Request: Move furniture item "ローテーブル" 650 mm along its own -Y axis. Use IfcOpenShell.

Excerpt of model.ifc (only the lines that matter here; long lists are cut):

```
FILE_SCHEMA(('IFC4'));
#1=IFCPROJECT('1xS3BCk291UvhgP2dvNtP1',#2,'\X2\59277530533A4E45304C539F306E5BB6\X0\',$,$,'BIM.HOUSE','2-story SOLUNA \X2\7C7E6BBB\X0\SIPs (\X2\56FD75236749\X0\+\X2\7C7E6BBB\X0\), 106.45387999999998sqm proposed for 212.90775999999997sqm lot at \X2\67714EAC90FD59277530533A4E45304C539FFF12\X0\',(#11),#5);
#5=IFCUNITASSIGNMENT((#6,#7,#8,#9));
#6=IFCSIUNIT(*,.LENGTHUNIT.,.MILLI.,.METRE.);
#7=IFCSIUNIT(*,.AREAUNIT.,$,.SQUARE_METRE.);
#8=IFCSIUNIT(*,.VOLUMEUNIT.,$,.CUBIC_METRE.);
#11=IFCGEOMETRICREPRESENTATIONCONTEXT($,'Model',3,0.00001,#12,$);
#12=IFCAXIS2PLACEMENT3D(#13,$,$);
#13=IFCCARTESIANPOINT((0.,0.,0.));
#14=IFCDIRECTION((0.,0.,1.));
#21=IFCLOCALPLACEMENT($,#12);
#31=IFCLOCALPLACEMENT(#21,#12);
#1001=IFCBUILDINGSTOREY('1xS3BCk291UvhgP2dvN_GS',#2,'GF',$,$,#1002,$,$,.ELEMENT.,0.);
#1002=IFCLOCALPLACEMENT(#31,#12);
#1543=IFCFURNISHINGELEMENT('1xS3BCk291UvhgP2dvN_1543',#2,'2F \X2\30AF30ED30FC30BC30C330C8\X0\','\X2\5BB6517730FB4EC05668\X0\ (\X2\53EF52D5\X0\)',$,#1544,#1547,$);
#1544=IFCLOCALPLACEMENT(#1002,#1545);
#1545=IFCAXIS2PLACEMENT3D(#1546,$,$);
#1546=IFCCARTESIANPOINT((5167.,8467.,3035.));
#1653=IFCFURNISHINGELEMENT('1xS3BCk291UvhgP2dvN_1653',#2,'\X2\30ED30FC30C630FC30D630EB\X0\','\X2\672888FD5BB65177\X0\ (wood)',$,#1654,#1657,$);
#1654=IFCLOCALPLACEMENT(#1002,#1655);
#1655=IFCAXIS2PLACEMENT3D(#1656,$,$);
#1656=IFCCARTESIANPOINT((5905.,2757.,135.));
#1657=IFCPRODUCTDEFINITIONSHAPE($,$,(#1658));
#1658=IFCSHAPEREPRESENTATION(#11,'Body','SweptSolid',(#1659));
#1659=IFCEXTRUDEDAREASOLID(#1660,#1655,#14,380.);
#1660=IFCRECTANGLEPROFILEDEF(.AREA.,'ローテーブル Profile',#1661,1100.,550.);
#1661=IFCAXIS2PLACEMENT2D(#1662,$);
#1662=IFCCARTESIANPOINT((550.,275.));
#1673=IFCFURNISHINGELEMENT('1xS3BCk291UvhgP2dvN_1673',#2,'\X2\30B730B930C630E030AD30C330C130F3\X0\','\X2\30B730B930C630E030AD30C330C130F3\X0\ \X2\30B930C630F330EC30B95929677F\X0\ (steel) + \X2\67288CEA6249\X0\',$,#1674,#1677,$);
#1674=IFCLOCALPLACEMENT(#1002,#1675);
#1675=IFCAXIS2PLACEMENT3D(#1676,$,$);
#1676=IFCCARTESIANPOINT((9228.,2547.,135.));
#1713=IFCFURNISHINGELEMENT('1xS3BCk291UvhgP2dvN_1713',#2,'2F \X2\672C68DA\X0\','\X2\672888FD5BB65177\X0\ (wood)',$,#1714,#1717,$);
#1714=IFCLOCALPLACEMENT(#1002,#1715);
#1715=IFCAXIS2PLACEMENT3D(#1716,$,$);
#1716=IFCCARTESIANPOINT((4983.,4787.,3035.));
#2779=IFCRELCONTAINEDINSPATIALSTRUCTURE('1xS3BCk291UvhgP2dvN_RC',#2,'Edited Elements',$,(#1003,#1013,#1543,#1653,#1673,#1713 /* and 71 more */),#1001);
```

```python
import ifcopenshell
import ifcopenshell.api.geometry
import ifcopenshell.util.placement
import ifcopenshell.util.unit

model = ifcopenshell.open("model.ifc")
unit_scale = ifcopenshell.util.unit.calculate_unit_scale(model)

item = model.by_id(1653)
matrix = ifcopenshell.util.placement.get_local_placement(item.ObjectPlacement)
matrix[:3, 3] -= matrix[:3, 1] * 0.65 / unit_scale
ifcopenshell.api.geometry.edit_object_placement(model, product=item, matrix=matrix, is_si=False)

print(ifcopenshell.util.placement.get_local_placement(item.ObjectPlacement).round(3) + 0.0)

model.write("model_v2.ifc")
```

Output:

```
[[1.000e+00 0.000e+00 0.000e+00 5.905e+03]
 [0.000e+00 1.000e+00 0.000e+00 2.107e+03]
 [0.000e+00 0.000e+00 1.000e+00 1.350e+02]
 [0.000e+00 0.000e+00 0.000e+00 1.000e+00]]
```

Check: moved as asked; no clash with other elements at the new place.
